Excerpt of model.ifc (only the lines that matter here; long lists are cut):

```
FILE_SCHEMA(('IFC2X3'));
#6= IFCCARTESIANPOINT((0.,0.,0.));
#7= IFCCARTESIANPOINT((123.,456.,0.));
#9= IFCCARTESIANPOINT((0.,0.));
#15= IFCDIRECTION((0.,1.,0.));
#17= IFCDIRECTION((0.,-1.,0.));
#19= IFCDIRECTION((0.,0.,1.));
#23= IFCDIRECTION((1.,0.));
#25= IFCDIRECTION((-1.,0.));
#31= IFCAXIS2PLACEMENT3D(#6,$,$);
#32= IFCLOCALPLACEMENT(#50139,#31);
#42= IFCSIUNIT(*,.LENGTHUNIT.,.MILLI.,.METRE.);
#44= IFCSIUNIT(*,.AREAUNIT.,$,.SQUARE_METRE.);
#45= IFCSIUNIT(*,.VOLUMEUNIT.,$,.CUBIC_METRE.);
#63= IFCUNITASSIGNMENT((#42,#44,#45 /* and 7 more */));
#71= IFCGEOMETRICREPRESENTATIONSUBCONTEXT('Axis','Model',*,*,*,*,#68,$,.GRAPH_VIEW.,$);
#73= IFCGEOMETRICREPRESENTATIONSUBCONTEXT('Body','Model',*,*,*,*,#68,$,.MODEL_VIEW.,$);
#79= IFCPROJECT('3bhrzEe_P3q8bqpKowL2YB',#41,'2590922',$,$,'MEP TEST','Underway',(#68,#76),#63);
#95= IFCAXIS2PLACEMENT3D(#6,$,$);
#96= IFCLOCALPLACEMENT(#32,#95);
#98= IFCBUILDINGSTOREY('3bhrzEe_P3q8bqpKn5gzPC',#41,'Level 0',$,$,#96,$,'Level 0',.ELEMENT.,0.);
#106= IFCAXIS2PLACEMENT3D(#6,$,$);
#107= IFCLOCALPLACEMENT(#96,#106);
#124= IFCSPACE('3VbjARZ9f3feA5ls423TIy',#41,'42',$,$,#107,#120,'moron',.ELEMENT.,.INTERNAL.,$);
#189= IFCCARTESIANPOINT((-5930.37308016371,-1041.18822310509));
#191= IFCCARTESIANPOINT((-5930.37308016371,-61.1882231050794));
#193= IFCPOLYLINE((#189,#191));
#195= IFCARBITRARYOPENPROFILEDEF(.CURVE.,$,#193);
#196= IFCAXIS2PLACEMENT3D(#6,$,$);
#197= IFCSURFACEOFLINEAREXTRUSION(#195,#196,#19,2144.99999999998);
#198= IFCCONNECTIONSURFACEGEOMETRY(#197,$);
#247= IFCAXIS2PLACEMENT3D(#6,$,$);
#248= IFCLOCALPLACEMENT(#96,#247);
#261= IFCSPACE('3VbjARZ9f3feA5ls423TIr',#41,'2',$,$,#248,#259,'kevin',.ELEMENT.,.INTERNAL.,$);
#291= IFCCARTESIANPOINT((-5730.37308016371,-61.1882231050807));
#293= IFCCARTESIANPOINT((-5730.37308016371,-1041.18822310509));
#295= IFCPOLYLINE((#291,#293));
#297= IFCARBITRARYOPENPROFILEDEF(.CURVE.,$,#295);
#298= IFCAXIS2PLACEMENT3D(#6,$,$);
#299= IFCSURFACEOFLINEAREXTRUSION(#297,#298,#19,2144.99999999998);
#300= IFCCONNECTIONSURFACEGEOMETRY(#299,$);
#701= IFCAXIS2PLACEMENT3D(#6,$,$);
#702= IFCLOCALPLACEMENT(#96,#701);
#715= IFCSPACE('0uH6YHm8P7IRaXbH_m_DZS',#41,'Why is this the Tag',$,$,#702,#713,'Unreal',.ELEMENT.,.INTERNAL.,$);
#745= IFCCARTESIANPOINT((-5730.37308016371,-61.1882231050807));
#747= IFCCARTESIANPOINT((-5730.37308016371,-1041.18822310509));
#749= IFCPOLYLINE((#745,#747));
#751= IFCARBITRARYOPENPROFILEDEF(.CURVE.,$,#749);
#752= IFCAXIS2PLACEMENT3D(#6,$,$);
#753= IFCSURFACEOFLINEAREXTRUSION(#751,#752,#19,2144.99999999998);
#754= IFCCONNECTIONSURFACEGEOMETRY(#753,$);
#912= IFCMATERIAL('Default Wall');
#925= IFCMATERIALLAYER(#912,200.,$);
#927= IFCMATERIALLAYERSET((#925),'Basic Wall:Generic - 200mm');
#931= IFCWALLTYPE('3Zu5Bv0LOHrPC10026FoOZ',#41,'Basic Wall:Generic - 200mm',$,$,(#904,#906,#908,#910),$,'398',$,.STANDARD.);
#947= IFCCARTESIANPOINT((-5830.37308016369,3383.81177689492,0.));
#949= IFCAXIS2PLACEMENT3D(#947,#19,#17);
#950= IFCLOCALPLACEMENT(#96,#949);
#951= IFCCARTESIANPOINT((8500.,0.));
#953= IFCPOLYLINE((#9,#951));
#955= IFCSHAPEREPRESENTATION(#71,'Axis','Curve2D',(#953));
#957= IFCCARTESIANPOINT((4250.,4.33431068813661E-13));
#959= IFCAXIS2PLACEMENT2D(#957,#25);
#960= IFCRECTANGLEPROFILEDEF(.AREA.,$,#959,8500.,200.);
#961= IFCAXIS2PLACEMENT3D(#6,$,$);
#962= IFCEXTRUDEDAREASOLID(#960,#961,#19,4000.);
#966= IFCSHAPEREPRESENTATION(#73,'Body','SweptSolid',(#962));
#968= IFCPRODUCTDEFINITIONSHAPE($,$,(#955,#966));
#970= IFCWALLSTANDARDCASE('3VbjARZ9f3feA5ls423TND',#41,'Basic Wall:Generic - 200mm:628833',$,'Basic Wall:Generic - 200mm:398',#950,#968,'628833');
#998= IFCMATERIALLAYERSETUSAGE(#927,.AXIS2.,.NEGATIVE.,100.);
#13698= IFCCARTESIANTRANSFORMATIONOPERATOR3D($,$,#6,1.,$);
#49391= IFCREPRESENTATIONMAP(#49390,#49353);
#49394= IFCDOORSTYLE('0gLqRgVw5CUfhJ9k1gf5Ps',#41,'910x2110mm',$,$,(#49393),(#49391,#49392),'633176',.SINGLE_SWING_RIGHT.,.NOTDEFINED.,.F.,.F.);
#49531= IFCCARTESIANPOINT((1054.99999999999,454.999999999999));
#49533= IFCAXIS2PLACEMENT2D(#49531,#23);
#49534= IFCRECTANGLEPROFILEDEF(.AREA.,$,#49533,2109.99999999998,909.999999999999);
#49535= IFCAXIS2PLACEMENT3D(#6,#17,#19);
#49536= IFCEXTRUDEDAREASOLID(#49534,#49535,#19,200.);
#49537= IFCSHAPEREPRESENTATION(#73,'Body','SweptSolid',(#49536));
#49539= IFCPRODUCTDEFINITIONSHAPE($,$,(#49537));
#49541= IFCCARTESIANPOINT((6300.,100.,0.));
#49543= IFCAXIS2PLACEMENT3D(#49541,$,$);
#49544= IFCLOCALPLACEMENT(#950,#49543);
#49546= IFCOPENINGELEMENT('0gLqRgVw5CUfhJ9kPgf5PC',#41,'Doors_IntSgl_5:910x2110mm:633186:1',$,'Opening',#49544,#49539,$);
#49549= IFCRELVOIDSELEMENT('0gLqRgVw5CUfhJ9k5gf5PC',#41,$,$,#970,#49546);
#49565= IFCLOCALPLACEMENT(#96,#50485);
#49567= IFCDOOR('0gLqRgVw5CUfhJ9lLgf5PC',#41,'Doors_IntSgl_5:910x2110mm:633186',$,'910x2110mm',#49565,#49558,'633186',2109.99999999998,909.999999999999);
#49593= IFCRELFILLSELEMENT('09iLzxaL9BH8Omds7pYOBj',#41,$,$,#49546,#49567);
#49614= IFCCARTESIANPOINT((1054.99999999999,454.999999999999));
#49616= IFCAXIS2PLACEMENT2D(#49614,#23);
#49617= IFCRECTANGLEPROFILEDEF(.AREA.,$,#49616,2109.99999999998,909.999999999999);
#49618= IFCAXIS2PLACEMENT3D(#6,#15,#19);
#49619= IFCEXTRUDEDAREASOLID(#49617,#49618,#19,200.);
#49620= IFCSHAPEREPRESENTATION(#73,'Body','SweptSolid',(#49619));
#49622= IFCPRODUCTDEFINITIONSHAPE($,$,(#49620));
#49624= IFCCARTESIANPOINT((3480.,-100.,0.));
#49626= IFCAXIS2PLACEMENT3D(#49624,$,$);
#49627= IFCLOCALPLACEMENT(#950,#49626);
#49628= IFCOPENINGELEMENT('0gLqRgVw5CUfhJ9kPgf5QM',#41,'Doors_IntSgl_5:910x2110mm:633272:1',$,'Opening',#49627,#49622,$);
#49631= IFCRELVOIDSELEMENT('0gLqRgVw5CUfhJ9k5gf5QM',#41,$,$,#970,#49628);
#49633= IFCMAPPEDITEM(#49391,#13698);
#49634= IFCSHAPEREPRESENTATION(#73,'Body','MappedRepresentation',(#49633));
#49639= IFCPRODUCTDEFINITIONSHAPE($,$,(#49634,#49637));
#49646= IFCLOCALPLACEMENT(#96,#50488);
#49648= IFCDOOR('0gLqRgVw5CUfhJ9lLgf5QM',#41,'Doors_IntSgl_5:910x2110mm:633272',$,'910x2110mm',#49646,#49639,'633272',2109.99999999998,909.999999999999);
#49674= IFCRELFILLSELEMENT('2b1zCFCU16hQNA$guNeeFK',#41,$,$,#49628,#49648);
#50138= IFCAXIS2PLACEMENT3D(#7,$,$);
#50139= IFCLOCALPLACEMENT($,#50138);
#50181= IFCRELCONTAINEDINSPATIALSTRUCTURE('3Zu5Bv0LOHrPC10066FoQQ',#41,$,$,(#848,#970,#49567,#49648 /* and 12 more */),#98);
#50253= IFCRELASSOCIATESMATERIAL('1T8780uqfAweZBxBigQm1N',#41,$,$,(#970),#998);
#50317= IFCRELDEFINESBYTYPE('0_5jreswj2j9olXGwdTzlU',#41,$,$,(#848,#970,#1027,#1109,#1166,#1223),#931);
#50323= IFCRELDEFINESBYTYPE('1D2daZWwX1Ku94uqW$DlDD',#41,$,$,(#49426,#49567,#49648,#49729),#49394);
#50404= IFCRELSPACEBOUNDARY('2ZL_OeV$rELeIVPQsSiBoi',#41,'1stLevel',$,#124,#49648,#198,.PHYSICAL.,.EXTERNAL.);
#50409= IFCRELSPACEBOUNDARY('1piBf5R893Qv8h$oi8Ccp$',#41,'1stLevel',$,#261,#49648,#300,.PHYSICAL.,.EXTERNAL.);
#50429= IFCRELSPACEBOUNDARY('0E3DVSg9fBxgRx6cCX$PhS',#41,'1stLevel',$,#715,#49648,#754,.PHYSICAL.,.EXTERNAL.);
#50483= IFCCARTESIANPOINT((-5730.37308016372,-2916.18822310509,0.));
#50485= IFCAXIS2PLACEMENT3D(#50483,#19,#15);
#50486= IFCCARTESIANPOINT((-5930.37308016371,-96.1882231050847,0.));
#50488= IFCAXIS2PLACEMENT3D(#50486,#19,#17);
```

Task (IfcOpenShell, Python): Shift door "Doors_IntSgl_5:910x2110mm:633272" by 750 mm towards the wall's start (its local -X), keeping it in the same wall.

```python
import numpy as np
import ifcopenshell
import ifcopenshell.api.geometry
import ifcopenshell.util.placement
import ifcopenshell.util.unit

model = ifcopenshell.open("model.ifc")
unit_scale = ifcopenshell.util.unit.calculate_unit_scale(model)

door = model.by_id(49648)
opening = door.FillsVoids[0].RelatingOpeningElement
wall = opening.VoidsElements[0].RelatingBuildingElement

wall_matrix = ifcopenshell.util.placement.get_local_placement(wall.ObjectPlacement)
shift = wall_matrix[:3, 0] * -0.75 / unit_scale
before = ifcopenshell.util.placement.get_local_placement(door.ObjectPlacement)[:3, 3].copy()

# The door is not placed relative to its opening, so move both.
for product in (opening, door):
    matrix = ifcopenshell.util.placement.get_local_placement(product.ObjectPlacement)
    matrix[:3, 3] += shift
    ifcopenshell.api.geometry.edit_object_placement(model, product=product, matrix=matrix, is_si=False)

# Space boundary surfaces are stored in each space's coordinates; move them too.
for rel in door.ProvidesBoundaries:
    if not rel.ConnectionGeometry:
        continue
    surface = rel.ConnectionGeometry.SurfaceOnRelatingElement
    space_matrix = ifcopenshell.util.placement.get_local_placement(rel.RelatingSpace.ObjectPlacement)
    point = np.array(surface.Position.Location.Coordinates) + space_matrix[:3, :3].T @ shift
    surface.Position = model.createIfcAxis2Placement3D(
        model.createIfcCartesianPoint(point.tolist()), surface.Position.Axis, surface.Position.RefDirection
    )

after = ifcopenshell.util.placement.get_local_placement(door.ObjectPlacement)[:3, 3]
print("door moved by", (after - before).round(3) + 0.0)

model.write("model_rev.ifc")
```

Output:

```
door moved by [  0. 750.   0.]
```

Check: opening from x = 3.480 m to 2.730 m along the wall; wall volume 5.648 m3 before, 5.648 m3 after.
